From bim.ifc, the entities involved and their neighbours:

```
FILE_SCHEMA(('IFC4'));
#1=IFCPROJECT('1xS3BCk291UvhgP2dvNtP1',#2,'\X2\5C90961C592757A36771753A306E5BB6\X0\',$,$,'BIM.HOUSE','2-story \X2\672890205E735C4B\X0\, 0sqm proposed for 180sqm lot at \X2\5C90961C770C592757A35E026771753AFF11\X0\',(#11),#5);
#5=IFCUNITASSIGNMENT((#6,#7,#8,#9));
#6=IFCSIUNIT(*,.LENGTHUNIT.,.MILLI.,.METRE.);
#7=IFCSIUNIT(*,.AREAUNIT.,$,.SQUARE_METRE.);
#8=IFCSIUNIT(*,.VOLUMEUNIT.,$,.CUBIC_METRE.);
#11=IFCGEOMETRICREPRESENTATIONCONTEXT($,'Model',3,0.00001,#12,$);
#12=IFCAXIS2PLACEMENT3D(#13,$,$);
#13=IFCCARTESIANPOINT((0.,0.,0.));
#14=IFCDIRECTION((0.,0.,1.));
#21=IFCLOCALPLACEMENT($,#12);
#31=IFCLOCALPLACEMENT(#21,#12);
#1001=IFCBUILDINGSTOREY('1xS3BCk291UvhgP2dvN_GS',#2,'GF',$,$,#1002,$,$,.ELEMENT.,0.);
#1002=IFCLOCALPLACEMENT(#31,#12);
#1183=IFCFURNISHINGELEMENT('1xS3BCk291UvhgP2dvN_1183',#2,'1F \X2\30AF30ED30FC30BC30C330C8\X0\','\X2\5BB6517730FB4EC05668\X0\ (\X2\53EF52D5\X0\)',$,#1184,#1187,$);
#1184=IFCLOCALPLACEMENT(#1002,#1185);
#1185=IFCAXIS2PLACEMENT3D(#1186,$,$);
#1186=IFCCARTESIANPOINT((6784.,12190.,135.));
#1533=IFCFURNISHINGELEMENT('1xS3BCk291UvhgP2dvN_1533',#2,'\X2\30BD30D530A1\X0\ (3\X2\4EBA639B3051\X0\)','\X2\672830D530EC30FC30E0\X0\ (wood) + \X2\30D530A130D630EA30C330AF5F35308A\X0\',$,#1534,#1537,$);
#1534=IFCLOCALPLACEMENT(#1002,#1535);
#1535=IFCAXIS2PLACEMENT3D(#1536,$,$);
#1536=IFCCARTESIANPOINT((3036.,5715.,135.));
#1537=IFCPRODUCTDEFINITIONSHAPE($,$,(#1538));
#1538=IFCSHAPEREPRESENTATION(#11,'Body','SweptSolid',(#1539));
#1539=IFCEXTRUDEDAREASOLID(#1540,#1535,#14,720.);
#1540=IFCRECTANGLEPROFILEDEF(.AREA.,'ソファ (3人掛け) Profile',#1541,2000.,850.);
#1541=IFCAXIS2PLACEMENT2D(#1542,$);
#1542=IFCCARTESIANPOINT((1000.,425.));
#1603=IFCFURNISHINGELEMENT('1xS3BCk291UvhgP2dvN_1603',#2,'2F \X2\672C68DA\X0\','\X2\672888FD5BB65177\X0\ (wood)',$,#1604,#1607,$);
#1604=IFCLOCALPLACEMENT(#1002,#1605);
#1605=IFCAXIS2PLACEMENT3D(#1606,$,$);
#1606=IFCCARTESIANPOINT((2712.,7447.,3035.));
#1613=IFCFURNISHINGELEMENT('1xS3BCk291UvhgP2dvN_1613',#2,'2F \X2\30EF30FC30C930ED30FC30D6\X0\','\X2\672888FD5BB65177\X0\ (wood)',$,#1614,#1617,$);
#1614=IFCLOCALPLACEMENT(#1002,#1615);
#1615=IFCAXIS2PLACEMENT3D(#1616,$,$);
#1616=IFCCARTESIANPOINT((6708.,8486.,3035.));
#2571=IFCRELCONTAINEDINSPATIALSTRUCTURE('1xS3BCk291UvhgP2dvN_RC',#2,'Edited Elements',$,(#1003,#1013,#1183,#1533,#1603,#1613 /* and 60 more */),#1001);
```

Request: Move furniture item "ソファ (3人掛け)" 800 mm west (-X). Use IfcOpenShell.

```python
import ifcopenshell
import ifcopenshell.api.geometry
import ifcopenshell.util.placement
import ifcopenshell.util.unit

model = ifcopenshell.open("bim.ifc")
unit_scale = ifcopenshell.util.unit.calculate_unit_scale(model)

item = model.by_guid("1xS3BCk291UvhgP2dvN_1533")
matrix = ifcopenshell.util.placement.get_local_placement(item.ObjectPlacement)
matrix[0, 3] -= 0.8 / unit_scale
ifcopenshell.api.geometry.edit_object_placement(model, product=item, matrix=matrix, is_si=False)

print(ifcopenshell.util.placement.get_local_placement(item.ObjectPlacement).round(3) + 0.0)

model.write("bim_rev.ifc")
```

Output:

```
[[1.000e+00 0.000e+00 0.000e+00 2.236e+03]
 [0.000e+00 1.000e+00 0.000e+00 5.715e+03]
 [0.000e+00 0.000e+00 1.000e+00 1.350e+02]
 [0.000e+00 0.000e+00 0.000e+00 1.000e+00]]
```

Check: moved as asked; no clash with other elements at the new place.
